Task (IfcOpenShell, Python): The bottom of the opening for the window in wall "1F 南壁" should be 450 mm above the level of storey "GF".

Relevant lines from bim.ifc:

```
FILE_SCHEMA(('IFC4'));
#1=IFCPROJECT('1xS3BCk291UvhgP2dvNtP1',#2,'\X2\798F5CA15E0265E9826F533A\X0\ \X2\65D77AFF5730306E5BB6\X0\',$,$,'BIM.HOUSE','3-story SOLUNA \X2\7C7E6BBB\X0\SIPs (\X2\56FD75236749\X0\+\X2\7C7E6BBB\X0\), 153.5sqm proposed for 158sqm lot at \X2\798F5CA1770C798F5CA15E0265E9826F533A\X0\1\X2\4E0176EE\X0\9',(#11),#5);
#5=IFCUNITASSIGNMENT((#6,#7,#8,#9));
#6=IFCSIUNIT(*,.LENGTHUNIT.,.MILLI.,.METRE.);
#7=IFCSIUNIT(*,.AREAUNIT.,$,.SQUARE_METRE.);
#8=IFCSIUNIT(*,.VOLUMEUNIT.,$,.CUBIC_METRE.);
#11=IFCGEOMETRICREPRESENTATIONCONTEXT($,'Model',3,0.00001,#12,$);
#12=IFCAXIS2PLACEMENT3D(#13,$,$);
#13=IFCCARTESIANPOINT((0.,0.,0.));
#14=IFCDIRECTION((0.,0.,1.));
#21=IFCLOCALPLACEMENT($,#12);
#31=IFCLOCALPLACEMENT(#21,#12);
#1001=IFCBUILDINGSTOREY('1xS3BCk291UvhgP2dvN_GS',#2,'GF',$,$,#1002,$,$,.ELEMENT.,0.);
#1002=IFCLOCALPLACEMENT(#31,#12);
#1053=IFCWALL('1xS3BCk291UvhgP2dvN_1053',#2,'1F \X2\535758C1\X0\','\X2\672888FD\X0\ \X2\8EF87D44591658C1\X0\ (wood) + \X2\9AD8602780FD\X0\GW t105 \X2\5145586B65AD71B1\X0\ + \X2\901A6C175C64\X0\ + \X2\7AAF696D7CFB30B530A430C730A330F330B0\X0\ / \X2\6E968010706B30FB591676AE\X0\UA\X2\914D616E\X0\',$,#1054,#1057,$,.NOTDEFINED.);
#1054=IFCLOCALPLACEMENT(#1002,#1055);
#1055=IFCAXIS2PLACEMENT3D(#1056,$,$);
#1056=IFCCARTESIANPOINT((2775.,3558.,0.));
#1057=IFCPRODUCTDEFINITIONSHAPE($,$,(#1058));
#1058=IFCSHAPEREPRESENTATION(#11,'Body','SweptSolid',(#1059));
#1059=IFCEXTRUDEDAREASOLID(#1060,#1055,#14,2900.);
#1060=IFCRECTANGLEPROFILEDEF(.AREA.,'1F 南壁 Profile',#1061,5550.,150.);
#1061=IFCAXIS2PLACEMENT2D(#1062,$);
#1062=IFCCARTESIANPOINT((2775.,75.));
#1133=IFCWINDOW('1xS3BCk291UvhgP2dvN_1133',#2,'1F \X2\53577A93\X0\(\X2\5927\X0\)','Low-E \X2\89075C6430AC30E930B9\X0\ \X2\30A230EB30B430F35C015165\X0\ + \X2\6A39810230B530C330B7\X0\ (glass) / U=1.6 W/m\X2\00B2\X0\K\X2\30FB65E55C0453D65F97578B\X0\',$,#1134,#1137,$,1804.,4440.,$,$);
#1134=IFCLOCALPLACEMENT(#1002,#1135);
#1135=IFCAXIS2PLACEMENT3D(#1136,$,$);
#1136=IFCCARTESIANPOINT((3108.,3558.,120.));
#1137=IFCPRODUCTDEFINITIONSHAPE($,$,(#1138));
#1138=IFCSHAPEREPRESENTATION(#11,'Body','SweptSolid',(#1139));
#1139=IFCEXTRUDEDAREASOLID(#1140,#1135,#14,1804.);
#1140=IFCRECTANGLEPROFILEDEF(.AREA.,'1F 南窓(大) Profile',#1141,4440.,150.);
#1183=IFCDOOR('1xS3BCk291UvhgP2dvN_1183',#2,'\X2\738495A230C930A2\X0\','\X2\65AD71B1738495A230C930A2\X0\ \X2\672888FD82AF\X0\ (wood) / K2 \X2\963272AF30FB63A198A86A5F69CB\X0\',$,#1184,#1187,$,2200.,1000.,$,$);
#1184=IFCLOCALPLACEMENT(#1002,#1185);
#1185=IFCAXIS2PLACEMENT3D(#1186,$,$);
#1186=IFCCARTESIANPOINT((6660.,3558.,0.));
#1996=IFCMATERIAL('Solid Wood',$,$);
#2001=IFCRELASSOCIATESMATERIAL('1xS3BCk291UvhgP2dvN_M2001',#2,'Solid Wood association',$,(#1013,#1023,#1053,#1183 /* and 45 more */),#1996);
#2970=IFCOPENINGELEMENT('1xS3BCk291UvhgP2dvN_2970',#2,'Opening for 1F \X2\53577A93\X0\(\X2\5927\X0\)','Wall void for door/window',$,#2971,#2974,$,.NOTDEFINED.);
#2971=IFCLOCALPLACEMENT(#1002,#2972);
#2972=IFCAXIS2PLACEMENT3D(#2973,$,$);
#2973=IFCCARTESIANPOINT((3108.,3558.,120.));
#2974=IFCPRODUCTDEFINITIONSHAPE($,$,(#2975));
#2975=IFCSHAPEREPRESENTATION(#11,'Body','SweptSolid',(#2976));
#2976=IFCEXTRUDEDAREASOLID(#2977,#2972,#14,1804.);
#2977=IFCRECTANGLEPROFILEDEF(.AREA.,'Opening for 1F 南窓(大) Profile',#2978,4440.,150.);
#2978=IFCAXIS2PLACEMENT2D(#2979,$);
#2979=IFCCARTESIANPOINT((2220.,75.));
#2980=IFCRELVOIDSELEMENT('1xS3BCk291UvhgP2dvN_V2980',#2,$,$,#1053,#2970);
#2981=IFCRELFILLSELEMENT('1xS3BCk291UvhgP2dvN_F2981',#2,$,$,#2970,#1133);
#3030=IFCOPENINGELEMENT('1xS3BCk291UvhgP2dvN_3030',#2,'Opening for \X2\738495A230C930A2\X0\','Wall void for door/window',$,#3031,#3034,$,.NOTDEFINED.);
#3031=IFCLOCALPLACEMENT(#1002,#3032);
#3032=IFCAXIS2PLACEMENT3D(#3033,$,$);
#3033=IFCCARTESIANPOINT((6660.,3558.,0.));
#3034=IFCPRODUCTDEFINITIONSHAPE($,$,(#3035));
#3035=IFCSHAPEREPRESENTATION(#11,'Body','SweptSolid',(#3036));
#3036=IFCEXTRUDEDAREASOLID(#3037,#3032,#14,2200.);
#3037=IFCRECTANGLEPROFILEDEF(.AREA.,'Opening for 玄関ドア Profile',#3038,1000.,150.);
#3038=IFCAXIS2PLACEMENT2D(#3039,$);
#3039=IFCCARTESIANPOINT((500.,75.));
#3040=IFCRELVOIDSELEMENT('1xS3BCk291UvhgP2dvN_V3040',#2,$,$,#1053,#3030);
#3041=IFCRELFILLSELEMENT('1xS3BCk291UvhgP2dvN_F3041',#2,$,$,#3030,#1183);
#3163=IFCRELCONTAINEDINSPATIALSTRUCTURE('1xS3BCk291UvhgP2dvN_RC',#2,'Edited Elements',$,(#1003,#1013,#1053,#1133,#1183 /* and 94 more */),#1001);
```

```python
import numpy as np
import ifcopenshell
import ifcopenshell.api.geometry
import ifcopenshell.geom
import ifcopenshell.util.element
import ifcopenshell.util.placement
import ifcopenshell.util.shape
import ifcopenshell.util.unit

model = ifcopenshell.open("bim.ifc")
unit_scale = ifcopenshell.util.unit.calculate_unit_scale(model)

window = model.by_id(1133)
opening = window.FillsVoids[0].RelatingOpeningElement
storey = ifcopenshell.util.element.get_container(window, ifc_class="IfcBuildingStorey")
level = ifcopenshell.util.placement.get_local_placement(storey.ObjectPlacement)[2, 3]

# The opening's origin need not be at the sill, so measure its lowest point.
shape = ifcopenshell.geom.create_shape(ifcopenshell.geom.settings(), opening)
bottom = ifcopenshell.util.shape.get_shape_bottom_elevation(shape, shape.geometry) / unit_scale
dz = level + 0.45 / unit_scale - bottom

shift = np.array([0.0, 0.0, dz])
# The window is not placed relative to its opening, so move both.
for product in (opening, window):
    matrix = ifcopenshell.util.placement.get_local_placement(product.ObjectPlacement)
    matrix[:3, 3] += shift
    ifcopenshell.api.geometry.edit_object_placement(model, product=product, matrix=matrix, is_si=False)

print(f"moved by {dz * unit_scale:+.3f} m")

model.write("bim_updated.ifc")
```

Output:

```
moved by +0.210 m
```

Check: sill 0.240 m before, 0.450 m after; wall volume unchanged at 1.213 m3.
